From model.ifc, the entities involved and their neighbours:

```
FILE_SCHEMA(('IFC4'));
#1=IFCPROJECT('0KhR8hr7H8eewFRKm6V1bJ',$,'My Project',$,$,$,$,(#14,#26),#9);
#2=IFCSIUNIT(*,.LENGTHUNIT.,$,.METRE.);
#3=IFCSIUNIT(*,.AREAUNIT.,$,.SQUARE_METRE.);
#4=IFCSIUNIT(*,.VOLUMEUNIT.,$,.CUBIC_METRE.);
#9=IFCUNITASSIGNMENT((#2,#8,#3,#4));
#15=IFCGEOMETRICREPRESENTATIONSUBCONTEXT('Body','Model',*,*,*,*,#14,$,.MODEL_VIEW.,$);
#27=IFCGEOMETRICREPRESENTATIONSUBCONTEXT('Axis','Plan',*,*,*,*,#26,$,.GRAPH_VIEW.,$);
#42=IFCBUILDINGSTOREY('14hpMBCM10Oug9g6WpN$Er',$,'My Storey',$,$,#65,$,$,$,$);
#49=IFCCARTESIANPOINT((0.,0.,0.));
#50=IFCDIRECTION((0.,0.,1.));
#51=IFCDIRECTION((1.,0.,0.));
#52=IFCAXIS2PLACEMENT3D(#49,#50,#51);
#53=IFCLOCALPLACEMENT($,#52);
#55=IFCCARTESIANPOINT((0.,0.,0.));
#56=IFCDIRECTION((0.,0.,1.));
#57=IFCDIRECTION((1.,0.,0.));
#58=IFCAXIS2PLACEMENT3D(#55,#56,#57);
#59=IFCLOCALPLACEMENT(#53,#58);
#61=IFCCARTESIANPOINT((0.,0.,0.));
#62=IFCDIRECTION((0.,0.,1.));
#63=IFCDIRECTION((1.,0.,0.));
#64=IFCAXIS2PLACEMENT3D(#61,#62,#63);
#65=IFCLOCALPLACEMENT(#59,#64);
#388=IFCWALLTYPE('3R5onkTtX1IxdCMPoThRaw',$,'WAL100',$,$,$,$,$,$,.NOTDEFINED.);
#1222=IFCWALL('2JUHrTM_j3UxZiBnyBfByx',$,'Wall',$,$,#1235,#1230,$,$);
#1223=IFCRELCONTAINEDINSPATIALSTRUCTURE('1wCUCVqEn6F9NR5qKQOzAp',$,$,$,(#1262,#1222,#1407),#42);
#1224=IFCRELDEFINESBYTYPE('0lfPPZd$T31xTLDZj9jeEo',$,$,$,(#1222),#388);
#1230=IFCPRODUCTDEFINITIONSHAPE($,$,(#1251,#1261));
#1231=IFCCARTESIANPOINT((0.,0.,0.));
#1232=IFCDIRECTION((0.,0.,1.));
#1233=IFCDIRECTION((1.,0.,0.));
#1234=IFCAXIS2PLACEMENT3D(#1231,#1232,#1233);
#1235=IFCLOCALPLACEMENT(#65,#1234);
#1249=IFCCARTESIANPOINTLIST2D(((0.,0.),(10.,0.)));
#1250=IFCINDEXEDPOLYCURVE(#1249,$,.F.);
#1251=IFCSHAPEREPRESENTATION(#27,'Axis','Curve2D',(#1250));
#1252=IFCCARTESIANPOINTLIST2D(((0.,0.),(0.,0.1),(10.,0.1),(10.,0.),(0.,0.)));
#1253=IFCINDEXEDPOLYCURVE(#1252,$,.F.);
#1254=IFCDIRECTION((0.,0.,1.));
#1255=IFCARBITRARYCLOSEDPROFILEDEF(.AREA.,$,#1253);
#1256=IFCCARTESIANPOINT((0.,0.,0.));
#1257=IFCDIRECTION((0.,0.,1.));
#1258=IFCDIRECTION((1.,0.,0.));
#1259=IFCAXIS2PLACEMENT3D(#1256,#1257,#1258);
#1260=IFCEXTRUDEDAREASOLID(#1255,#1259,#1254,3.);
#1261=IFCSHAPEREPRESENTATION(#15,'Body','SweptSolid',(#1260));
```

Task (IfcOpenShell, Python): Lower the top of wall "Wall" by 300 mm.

```python
import ifcopenshell
import ifcopenshell.geom
import ifcopenshell.util.representation
import ifcopenshell.util.shape

model = ifcopenshell.open("model.ifc")
settings = ifcopenshell.geom.settings()


def volume(element):
    """Net volume in cubic metres, openings subtracted."""
    shape = ifcopenshell.geom.create_shape(settings, element)
    return ifcopenshell.util.shape.get_volume(shape.geometry)


wall = model.by_guid("2JUHrTM_j3UxZiBnyBfByx")
before = volume(wall)

body = ifcopenshell.util.representation.get_representation(wall, "Model", "Body")
solid = body.Items[0]
old_height = solid.Depth
solid.Depth -= 0.3
after = volume(wall)

print(f"height {old_height:g} -> {solid.Depth:g}, volume {before:.3f} -> {after:.3f} m3")

model.write("model_rev.ifc")
```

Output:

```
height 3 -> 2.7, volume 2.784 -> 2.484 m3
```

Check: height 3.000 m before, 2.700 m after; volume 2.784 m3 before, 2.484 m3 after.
